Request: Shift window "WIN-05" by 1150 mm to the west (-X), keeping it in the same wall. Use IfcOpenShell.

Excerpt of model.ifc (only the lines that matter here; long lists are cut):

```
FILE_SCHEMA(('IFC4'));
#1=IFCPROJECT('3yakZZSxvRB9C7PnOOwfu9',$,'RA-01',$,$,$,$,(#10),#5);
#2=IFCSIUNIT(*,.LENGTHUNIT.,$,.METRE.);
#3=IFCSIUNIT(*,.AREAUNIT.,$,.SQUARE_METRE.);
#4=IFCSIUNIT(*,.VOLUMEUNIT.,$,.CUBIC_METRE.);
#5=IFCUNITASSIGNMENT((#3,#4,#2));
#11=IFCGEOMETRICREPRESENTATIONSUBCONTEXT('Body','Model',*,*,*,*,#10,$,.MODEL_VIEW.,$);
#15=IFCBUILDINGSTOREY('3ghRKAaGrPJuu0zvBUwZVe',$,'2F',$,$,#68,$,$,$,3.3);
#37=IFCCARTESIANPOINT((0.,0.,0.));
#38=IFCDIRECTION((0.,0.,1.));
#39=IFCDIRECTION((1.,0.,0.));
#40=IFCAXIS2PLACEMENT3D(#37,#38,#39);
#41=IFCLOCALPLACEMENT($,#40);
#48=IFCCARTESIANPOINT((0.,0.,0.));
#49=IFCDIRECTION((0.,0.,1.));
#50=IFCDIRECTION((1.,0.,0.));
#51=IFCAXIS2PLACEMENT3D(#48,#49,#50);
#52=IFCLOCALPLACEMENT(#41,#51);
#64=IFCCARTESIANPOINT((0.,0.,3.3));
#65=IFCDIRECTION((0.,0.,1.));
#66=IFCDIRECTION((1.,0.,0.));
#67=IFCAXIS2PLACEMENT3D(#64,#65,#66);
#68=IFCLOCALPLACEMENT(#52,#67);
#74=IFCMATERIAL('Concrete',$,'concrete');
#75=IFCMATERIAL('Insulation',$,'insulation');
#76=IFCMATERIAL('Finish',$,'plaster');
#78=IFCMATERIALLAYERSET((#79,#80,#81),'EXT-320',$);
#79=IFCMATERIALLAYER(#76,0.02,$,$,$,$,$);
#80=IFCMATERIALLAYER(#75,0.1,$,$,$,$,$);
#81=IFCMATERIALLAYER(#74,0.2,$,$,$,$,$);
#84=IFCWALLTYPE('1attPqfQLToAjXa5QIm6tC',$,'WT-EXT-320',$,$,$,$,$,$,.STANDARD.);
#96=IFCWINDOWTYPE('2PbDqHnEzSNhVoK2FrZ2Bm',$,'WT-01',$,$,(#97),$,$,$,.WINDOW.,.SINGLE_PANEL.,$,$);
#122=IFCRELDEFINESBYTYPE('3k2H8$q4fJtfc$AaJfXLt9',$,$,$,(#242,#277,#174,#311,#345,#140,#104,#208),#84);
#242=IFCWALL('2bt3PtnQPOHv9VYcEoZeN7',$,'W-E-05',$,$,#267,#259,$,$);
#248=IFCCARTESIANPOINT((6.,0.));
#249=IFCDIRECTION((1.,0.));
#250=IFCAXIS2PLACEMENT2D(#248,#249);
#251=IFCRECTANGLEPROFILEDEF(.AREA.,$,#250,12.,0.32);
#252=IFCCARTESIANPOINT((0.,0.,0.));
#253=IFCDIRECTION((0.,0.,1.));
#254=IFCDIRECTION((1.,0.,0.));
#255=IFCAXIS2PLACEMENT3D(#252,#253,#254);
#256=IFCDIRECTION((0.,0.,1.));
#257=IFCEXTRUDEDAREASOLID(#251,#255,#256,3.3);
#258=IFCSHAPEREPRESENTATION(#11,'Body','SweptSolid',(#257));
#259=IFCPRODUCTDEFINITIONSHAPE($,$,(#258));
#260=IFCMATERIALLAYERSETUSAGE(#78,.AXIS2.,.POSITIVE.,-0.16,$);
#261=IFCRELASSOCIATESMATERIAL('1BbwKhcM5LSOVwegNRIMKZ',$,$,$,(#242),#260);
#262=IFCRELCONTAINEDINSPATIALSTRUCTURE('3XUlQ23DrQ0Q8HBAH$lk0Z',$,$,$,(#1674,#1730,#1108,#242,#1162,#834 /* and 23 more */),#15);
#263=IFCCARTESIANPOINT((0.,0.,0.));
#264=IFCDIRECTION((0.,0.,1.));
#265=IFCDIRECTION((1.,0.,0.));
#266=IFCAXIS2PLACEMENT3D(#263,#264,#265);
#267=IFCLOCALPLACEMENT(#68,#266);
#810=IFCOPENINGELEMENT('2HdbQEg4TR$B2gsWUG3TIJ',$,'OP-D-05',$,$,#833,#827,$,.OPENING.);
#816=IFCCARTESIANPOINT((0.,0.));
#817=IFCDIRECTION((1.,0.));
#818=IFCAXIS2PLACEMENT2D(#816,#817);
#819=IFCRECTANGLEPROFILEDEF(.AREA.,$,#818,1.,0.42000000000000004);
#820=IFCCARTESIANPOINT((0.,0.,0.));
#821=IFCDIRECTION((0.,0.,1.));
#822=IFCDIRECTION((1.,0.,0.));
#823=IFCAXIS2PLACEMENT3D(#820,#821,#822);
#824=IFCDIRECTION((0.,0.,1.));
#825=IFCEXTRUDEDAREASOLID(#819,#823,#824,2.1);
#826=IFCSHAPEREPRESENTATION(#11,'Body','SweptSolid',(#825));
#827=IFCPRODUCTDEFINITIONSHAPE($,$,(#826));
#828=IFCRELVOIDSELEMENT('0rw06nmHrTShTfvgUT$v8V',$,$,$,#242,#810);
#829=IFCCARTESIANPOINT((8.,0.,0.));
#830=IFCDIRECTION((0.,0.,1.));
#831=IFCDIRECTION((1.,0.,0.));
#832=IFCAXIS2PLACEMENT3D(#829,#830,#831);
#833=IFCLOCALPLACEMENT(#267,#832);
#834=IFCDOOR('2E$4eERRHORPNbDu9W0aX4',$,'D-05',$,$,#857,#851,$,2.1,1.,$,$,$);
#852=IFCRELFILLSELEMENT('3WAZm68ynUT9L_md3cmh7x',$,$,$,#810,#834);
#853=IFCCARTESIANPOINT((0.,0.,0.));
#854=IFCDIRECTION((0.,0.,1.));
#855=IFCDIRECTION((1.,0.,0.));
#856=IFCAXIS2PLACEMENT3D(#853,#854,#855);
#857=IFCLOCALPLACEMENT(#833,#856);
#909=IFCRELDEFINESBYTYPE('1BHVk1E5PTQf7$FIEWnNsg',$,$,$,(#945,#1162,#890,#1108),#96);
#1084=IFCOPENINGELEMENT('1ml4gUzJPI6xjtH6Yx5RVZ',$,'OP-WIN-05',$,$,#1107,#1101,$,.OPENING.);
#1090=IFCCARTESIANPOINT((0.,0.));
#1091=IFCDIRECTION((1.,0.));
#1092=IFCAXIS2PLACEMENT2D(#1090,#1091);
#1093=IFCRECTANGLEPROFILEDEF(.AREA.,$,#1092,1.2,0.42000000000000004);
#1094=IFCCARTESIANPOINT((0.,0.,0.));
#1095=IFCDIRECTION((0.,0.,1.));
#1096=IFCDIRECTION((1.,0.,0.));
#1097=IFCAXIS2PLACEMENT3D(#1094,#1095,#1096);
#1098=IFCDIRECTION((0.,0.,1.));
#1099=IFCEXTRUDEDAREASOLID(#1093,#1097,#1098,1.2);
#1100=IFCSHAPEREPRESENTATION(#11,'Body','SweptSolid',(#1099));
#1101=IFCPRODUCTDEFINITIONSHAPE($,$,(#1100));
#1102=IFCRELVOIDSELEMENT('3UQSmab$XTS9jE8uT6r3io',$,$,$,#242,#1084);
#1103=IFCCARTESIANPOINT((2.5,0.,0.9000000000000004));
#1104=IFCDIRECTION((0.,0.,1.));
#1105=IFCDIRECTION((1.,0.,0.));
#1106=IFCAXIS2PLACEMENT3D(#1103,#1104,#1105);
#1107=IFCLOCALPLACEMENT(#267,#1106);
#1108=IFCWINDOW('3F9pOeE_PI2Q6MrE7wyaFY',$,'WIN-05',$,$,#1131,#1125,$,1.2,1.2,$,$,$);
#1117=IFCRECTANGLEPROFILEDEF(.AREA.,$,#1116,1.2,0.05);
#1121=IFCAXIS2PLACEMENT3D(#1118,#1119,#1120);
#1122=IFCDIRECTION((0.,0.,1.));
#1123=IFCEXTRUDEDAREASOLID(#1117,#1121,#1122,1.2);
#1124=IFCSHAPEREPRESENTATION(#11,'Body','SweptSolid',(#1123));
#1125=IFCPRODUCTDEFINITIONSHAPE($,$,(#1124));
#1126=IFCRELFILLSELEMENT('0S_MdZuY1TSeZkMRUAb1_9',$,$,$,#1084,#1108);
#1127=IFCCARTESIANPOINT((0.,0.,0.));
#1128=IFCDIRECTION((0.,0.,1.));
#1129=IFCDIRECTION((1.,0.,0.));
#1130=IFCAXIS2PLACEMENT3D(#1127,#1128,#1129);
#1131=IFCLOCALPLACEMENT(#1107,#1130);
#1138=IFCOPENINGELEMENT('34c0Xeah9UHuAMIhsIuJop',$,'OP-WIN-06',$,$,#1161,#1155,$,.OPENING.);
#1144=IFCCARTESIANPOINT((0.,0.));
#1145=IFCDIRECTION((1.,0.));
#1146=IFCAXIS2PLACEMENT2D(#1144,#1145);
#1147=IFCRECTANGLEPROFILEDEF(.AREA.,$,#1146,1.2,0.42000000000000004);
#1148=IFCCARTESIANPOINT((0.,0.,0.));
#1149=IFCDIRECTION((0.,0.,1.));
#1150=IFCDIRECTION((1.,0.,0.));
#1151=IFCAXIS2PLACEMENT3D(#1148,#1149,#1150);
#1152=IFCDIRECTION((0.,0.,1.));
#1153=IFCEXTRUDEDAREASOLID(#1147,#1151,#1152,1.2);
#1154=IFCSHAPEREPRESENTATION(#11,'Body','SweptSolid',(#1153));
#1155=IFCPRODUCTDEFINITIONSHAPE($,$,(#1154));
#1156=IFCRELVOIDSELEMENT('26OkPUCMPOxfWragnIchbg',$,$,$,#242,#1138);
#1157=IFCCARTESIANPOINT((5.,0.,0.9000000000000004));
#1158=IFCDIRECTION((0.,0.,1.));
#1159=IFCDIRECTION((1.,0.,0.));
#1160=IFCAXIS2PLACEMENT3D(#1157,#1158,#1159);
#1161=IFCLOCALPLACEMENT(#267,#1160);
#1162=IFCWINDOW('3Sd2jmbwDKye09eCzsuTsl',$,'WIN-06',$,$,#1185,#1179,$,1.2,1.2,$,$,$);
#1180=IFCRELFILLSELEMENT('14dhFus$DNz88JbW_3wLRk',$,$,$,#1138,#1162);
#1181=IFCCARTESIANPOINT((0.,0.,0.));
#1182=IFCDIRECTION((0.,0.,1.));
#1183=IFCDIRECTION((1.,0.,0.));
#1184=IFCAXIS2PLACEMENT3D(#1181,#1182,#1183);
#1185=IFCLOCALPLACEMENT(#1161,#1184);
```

```python
import ifcopenshell
import ifcopenshell.api.geometry
import ifcopenshell.util.placement
import ifcopenshell.util.unit

model = ifcopenshell.open("model.ifc")
unit_scale = ifcopenshell.util.unit.calculate_unit_scale(model)

window = model.by_id(1108)
opening = window.FillsVoids[0].RelatingOpeningElement
wall = opening.VoidsElements[0].RelatingBuildingElement

wall_matrix = ifcopenshell.util.placement.get_local_placement(wall.ObjectPlacement)
shift = wall_matrix[:3, 0] * -1.15 / unit_scale
before = ifcopenshell.util.placement.get_local_placement(window.ObjectPlacement)[:3, 3].copy()

# The window is placed relative to its opening, so it follows when the opening moves.
matrix = ifcopenshell.util.placement.get_local_placement(opening.ObjectPlacement)
matrix[:3, 3] += shift
ifcopenshell.api.geometry.edit_object_placement(
    model, product=opening, matrix=matrix, is_si=False, should_transform_children=True
)

after = ifcopenshell.util.placement.get_local_placement(window.ObjectPlacement)[:3, 3]
print("window moved by", (after - before).round(3) + 0.0)

model.write("model_rev.ifc")
```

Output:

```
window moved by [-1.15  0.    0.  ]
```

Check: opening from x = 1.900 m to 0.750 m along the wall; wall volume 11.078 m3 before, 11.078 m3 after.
